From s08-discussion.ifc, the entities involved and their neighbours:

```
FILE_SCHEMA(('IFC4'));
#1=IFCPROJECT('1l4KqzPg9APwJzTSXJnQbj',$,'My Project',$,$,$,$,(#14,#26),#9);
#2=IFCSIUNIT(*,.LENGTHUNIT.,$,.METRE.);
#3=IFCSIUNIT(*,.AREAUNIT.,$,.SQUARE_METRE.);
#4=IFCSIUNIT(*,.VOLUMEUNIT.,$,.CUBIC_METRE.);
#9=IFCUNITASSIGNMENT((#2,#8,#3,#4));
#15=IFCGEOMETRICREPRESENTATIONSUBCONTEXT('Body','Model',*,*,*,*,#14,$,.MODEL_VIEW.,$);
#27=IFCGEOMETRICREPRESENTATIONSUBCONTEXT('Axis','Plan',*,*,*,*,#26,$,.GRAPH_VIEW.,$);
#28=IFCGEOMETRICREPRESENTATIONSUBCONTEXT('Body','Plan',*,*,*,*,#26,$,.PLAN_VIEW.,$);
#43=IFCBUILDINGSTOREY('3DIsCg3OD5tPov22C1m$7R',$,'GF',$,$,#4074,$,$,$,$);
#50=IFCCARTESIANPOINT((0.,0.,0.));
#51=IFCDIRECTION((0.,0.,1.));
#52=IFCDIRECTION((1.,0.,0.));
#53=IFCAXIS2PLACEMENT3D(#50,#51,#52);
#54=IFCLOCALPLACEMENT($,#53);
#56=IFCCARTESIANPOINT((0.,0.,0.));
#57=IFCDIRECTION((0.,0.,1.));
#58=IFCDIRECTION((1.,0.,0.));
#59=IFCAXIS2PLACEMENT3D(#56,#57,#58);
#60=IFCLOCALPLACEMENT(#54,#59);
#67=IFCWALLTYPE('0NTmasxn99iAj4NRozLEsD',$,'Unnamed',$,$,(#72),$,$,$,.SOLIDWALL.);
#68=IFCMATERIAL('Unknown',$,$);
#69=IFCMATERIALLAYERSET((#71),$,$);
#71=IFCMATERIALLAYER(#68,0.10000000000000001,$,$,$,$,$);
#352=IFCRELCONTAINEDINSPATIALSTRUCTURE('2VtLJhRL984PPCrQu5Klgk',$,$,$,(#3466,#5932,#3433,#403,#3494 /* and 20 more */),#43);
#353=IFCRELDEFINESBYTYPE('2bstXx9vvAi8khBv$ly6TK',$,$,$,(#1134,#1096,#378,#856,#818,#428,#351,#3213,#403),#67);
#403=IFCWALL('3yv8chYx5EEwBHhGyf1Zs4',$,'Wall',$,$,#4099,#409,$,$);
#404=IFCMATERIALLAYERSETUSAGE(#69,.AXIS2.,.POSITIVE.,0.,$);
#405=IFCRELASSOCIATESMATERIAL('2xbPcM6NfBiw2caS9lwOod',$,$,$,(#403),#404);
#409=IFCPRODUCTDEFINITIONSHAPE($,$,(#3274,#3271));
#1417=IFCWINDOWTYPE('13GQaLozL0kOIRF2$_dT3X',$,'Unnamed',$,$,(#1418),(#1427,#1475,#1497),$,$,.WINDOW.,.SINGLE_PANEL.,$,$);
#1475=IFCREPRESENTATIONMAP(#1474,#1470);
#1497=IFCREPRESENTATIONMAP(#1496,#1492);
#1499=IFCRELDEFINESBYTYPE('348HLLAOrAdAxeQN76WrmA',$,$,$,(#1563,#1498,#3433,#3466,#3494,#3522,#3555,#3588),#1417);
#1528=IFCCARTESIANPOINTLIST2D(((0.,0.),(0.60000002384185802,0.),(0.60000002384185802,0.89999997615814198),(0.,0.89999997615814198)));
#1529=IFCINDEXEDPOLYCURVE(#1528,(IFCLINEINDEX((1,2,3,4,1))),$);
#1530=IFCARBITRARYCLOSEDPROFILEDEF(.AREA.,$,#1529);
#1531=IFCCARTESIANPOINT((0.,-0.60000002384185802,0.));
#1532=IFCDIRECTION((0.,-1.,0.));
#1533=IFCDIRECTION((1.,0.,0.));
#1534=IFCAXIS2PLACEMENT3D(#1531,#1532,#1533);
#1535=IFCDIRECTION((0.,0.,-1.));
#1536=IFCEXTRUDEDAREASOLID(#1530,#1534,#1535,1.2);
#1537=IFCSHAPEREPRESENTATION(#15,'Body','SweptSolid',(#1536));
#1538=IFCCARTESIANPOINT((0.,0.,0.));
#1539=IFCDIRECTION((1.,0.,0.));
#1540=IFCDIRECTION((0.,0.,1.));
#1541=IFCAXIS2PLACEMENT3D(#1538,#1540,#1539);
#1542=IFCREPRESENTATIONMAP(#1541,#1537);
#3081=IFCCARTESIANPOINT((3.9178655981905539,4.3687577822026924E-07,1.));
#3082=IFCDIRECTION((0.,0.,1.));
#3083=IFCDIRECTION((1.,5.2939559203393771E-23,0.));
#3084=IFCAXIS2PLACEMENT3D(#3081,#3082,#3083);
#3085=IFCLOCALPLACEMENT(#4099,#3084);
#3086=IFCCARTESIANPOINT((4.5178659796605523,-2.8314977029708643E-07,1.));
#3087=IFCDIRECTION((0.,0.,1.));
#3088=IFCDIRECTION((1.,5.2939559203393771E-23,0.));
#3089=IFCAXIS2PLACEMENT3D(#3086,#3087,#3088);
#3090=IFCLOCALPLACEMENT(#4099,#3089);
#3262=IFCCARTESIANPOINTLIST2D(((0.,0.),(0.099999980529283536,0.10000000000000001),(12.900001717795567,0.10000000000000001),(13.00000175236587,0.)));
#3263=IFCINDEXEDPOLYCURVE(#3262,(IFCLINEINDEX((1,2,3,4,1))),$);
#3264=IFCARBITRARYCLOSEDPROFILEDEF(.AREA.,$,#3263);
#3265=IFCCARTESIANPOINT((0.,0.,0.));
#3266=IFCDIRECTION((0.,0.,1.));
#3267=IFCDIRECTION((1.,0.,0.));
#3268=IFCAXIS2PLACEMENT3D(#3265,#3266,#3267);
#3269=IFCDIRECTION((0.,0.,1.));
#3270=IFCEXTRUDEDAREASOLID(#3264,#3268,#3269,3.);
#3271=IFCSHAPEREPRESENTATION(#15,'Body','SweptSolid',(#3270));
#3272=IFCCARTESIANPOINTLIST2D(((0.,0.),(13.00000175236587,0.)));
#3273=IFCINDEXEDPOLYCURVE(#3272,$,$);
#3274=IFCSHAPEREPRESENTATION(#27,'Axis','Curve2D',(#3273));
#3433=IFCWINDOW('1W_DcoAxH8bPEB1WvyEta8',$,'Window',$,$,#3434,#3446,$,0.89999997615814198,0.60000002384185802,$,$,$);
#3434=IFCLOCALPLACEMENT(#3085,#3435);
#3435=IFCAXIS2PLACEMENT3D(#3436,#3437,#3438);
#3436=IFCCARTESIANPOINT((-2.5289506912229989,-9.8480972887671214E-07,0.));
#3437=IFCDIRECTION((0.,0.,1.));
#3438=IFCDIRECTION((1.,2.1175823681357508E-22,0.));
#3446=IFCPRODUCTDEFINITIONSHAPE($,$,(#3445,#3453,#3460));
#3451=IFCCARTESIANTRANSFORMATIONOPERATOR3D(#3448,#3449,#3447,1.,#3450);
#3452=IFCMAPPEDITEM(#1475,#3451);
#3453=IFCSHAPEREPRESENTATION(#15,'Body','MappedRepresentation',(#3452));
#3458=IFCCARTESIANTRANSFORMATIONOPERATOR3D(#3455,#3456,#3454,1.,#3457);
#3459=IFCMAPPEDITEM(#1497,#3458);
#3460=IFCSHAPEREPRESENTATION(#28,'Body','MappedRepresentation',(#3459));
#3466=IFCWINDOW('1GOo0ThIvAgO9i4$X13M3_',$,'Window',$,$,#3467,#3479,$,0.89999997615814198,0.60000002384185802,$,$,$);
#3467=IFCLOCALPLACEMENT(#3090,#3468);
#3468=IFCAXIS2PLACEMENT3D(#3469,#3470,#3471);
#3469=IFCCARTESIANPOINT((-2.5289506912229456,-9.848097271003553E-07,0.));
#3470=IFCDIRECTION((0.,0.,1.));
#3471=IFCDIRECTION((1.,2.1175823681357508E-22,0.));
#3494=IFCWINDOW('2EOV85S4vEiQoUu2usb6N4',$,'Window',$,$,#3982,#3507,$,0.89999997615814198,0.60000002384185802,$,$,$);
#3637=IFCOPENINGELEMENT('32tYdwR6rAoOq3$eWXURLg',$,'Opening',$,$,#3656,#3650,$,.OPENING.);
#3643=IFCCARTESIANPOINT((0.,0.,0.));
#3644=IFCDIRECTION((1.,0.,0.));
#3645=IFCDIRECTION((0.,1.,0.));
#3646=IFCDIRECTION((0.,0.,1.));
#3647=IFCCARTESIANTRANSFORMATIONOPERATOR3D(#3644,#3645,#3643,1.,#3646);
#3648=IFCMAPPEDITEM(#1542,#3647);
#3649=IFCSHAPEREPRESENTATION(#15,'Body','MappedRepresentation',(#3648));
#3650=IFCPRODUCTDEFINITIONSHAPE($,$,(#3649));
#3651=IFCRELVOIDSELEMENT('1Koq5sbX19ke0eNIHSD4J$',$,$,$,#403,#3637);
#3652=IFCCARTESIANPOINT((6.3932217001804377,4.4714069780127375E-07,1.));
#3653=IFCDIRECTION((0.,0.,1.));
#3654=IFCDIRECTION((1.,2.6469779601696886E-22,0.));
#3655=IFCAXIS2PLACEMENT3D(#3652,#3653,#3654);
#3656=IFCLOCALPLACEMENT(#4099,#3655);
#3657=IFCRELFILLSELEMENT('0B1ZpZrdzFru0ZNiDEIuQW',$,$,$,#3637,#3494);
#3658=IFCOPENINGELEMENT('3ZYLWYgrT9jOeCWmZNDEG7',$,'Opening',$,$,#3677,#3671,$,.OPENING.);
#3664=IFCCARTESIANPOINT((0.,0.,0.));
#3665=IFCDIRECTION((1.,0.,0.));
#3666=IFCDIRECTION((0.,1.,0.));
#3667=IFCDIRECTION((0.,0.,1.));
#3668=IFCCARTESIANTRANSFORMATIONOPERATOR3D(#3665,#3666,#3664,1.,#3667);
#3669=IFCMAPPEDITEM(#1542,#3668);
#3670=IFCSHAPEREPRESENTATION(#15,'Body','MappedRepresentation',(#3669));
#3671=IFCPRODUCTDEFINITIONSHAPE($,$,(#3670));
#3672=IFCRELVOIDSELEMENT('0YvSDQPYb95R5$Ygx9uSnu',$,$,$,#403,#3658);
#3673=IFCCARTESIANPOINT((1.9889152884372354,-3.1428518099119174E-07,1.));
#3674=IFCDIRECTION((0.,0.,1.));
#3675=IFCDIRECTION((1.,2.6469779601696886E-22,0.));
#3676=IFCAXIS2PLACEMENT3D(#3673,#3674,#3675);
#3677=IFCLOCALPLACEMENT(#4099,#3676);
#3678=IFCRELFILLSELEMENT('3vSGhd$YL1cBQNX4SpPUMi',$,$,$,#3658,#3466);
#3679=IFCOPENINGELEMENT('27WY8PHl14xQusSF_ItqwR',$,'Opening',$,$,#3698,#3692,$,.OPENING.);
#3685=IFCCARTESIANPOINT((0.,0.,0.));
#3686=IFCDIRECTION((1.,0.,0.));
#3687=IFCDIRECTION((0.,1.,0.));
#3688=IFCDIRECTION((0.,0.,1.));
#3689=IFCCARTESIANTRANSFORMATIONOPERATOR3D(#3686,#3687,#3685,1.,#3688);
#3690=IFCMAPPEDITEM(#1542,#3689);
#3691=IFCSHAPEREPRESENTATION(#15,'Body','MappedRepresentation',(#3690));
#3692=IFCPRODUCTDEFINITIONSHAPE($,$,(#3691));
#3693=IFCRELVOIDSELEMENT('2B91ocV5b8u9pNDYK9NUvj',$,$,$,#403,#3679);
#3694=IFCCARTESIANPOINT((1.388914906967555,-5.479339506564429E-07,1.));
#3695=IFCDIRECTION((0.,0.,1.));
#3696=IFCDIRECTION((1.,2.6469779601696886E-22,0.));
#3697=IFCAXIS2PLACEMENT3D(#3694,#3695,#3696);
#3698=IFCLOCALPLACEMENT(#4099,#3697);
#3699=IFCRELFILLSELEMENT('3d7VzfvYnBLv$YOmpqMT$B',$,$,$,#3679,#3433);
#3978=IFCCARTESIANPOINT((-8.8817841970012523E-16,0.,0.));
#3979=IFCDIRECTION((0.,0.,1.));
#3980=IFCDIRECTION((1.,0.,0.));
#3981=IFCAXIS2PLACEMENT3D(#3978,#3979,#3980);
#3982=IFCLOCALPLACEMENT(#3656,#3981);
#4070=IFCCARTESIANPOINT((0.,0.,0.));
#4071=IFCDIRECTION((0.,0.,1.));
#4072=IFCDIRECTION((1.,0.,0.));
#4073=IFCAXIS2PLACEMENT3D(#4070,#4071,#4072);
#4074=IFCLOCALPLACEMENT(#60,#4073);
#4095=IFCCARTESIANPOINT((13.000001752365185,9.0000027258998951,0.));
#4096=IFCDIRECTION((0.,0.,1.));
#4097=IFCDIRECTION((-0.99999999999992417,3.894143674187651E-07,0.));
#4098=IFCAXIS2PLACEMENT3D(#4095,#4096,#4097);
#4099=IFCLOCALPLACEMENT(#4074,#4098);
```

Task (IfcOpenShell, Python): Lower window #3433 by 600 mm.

```python
import numpy as np
import ifcopenshell
import ifcopenshell.api.geometry
import ifcopenshell.util.placement
import ifcopenshell.util.unit

model = ifcopenshell.open("s08-discussion.ifc")
unit_scale = ifcopenshell.util.unit.calculate_unit_scale(model)

window = model.by_id(3433)
opening = window.FillsVoids[0].RelatingOpeningElement
dz = -0.6 / unit_scale

shift = np.array([0.0, 0.0, dz])
# The window is not placed relative to its opening, so move both.
for product in (opening, window):
    matrix = ifcopenshell.util.placement.get_local_placement(product.ObjectPlacement)
    matrix[:3, 3] += shift
    ifcopenshell.api.geometry.edit_object_placement(model, product=product, matrix=matrix, is_si=False)

print(f"moved by {dz * unit_scale:+.3f} m")

model.write("s08-discussion_updated.ifc")
```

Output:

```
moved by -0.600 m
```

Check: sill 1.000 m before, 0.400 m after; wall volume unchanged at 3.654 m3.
